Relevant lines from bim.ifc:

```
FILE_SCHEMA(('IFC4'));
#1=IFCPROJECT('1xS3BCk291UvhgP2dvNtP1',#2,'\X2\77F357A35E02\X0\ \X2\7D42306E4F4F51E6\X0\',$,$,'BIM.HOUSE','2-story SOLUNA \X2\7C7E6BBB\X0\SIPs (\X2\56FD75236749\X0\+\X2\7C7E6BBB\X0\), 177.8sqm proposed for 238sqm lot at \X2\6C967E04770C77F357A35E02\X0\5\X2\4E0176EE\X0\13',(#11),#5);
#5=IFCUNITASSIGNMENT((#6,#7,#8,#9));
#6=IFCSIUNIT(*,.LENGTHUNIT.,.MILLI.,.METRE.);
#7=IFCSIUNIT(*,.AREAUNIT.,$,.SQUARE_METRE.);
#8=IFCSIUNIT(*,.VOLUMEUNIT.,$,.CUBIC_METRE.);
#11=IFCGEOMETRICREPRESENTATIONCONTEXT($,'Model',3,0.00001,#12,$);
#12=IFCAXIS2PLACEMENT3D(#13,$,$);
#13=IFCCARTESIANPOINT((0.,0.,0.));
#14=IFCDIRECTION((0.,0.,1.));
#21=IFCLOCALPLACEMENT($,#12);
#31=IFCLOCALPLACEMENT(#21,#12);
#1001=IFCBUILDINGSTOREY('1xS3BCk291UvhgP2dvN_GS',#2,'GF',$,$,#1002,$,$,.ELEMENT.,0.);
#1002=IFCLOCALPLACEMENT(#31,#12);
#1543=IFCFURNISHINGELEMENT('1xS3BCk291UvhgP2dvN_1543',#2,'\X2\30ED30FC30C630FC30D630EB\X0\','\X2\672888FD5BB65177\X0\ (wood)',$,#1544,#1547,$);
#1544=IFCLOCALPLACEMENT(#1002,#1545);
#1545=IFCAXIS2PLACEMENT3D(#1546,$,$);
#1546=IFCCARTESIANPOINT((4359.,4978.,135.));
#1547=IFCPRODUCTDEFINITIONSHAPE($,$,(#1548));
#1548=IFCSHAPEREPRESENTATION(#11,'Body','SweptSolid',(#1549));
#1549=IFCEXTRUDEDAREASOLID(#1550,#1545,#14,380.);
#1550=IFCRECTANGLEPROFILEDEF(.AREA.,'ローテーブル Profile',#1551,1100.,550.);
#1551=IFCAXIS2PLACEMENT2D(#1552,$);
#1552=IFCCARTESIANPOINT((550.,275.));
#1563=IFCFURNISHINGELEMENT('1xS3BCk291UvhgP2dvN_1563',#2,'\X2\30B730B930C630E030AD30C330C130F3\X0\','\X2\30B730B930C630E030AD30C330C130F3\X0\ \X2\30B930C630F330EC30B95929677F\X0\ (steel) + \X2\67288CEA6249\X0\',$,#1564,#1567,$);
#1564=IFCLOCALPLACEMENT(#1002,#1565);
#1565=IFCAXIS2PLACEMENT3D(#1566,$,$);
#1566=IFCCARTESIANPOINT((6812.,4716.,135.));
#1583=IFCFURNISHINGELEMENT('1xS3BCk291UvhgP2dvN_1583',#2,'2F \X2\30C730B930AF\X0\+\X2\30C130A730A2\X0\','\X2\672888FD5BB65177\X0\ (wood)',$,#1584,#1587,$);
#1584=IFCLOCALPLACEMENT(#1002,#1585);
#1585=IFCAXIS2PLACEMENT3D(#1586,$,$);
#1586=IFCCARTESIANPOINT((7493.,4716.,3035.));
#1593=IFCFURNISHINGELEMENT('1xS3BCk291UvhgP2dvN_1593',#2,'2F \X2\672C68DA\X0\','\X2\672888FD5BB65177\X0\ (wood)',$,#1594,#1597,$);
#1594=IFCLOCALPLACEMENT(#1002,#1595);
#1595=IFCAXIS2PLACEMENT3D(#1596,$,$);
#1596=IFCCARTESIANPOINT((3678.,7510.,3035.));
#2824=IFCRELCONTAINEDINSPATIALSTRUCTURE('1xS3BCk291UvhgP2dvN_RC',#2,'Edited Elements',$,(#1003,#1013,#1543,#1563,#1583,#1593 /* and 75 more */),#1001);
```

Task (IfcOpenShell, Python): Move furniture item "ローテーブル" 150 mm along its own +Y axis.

```python
import ifcopenshell
import ifcopenshell.api.geometry
import ifcopenshell.util.placement
import ifcopenshell.util.unit

model = ifcopenshell.open("bim.ifc")
unit_scale = ifcopenshell.util.unit.calculate_unit_scale(model)

item = model.by_id(1543)
matrix = ifcopenshell.util.placement.get_local_placement(item.ObjectPlacement)
matrix[:3, 3] += matrix[:3, 1] * 0.15 / unit_scale
ifcopenshell.api.geometry.edit_object_placement(model, product=item, matrix=matrix, is_si=False)

print(ifcopenshell.util.placement.get_local_placement(item.ObjectPlacement).round(3) + 0.0)

model.write("bim_rev.ifc")
```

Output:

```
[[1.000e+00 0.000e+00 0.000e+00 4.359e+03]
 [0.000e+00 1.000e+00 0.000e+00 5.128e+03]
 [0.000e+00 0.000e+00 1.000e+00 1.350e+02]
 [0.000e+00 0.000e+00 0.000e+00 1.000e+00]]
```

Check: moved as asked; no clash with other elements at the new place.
